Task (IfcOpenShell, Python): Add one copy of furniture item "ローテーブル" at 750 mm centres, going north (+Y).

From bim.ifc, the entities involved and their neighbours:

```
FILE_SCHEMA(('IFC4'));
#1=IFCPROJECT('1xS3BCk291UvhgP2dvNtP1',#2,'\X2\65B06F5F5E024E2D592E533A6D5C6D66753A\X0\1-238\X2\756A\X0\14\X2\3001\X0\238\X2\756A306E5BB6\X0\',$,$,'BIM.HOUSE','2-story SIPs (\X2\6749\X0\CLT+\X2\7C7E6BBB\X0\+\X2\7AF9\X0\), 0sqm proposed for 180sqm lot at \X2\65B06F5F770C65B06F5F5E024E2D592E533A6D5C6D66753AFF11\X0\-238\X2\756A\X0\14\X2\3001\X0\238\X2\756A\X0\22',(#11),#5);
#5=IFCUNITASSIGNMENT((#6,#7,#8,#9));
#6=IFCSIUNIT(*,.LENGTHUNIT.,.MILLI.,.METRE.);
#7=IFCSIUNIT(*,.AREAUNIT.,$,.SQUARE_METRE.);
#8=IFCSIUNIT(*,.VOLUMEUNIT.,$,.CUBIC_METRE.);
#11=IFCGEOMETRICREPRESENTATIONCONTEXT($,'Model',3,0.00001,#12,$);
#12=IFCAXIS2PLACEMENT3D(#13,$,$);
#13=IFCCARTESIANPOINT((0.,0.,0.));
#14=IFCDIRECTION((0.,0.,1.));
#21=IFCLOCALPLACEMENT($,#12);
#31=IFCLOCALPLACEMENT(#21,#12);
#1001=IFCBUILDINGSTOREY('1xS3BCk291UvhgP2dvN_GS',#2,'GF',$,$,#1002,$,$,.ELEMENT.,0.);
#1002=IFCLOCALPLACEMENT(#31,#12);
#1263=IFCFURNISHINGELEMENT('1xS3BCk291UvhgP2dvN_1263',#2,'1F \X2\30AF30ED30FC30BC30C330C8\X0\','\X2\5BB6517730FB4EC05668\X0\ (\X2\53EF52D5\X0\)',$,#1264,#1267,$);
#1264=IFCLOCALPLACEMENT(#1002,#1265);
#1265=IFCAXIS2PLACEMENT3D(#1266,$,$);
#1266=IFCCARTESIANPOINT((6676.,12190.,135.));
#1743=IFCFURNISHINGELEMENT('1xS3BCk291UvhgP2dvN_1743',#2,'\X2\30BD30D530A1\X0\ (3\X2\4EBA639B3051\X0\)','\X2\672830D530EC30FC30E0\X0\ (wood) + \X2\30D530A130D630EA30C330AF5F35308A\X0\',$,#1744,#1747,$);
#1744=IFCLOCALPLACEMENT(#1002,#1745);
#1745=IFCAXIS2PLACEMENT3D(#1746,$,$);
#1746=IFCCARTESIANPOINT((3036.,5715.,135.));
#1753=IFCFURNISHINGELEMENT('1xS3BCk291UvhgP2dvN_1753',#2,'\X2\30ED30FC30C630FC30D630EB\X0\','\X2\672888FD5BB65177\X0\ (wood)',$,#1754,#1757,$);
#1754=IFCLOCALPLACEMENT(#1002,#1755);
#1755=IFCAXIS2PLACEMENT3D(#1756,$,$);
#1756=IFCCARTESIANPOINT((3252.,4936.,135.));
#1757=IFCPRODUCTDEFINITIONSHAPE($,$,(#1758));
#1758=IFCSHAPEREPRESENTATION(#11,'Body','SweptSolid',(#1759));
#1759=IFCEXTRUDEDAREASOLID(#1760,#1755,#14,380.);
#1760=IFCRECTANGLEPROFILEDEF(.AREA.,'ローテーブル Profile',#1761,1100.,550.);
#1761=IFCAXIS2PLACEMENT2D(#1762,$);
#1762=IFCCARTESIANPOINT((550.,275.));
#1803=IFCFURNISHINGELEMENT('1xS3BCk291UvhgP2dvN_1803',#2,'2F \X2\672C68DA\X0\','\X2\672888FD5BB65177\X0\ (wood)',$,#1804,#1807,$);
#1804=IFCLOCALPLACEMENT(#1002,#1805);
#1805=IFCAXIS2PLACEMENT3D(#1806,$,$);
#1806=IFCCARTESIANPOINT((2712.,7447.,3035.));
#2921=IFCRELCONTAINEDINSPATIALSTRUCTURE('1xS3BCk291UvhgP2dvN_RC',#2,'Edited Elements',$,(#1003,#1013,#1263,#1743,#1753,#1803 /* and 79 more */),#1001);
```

```python
import numpy as np
import ifcopenshell
import ifcopenshell.api.geometry
import ifcopenshell.api.root
import ifcopenshell.util.element
import ifcopenshell.util.placement
import ifcopenshell.util.unit

model = ifcopenshell.open("bim.ifc")
unit_scale = ifcopenshell.util.unit.calculate_unit_scale(model)


def reuse_history(source, copy):
    """copy_class also copies each property set's owner history, people and application; keep the originals."""
    for rel in copy.IsDefinedBy:
        if rel.is_a("IfcRelDefinesByProperties") and (history := rel.RelatingPropertyDefinition.OwnerHistory):
            rel.RelatingPropertyDefinition.OwnerHistory = source.OwnerHistory
            ifcopenshell.util.element.remove_deep2(model, history)


source = model.by_guid("1xS3BCk291UvhgP2dvN_1753")
base = ifcopenshell.util.placement.get_local_placement(source.ObjectPlacement)
step = np.array([0.0, 1.0, 0.0]) * 0.75 / unit_scale

for i in range(1, 2):
    copy = ifcopenshell.api.root.copy_class(model, product=source)
    copy.Representation = ifcopenshell.util.element.copy_deep(
        model, source.Representation, exclude=["IfcGeometricRepresentationContext", "IfcRepresentationMap"]
    )
    reuse_history(source, copy)
    matrix = base.copy()
    matrix[:3, 3] += i * step
    print("added at", matrix[:3, 3].round(3) + 0.0)
    ifcopenshell.api.geometry.edit_object_placement(model, product=copy, matrix=matrix, is_si=False)

model.write("bim_updated.ifc")
```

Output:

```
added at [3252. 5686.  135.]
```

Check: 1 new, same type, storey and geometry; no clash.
